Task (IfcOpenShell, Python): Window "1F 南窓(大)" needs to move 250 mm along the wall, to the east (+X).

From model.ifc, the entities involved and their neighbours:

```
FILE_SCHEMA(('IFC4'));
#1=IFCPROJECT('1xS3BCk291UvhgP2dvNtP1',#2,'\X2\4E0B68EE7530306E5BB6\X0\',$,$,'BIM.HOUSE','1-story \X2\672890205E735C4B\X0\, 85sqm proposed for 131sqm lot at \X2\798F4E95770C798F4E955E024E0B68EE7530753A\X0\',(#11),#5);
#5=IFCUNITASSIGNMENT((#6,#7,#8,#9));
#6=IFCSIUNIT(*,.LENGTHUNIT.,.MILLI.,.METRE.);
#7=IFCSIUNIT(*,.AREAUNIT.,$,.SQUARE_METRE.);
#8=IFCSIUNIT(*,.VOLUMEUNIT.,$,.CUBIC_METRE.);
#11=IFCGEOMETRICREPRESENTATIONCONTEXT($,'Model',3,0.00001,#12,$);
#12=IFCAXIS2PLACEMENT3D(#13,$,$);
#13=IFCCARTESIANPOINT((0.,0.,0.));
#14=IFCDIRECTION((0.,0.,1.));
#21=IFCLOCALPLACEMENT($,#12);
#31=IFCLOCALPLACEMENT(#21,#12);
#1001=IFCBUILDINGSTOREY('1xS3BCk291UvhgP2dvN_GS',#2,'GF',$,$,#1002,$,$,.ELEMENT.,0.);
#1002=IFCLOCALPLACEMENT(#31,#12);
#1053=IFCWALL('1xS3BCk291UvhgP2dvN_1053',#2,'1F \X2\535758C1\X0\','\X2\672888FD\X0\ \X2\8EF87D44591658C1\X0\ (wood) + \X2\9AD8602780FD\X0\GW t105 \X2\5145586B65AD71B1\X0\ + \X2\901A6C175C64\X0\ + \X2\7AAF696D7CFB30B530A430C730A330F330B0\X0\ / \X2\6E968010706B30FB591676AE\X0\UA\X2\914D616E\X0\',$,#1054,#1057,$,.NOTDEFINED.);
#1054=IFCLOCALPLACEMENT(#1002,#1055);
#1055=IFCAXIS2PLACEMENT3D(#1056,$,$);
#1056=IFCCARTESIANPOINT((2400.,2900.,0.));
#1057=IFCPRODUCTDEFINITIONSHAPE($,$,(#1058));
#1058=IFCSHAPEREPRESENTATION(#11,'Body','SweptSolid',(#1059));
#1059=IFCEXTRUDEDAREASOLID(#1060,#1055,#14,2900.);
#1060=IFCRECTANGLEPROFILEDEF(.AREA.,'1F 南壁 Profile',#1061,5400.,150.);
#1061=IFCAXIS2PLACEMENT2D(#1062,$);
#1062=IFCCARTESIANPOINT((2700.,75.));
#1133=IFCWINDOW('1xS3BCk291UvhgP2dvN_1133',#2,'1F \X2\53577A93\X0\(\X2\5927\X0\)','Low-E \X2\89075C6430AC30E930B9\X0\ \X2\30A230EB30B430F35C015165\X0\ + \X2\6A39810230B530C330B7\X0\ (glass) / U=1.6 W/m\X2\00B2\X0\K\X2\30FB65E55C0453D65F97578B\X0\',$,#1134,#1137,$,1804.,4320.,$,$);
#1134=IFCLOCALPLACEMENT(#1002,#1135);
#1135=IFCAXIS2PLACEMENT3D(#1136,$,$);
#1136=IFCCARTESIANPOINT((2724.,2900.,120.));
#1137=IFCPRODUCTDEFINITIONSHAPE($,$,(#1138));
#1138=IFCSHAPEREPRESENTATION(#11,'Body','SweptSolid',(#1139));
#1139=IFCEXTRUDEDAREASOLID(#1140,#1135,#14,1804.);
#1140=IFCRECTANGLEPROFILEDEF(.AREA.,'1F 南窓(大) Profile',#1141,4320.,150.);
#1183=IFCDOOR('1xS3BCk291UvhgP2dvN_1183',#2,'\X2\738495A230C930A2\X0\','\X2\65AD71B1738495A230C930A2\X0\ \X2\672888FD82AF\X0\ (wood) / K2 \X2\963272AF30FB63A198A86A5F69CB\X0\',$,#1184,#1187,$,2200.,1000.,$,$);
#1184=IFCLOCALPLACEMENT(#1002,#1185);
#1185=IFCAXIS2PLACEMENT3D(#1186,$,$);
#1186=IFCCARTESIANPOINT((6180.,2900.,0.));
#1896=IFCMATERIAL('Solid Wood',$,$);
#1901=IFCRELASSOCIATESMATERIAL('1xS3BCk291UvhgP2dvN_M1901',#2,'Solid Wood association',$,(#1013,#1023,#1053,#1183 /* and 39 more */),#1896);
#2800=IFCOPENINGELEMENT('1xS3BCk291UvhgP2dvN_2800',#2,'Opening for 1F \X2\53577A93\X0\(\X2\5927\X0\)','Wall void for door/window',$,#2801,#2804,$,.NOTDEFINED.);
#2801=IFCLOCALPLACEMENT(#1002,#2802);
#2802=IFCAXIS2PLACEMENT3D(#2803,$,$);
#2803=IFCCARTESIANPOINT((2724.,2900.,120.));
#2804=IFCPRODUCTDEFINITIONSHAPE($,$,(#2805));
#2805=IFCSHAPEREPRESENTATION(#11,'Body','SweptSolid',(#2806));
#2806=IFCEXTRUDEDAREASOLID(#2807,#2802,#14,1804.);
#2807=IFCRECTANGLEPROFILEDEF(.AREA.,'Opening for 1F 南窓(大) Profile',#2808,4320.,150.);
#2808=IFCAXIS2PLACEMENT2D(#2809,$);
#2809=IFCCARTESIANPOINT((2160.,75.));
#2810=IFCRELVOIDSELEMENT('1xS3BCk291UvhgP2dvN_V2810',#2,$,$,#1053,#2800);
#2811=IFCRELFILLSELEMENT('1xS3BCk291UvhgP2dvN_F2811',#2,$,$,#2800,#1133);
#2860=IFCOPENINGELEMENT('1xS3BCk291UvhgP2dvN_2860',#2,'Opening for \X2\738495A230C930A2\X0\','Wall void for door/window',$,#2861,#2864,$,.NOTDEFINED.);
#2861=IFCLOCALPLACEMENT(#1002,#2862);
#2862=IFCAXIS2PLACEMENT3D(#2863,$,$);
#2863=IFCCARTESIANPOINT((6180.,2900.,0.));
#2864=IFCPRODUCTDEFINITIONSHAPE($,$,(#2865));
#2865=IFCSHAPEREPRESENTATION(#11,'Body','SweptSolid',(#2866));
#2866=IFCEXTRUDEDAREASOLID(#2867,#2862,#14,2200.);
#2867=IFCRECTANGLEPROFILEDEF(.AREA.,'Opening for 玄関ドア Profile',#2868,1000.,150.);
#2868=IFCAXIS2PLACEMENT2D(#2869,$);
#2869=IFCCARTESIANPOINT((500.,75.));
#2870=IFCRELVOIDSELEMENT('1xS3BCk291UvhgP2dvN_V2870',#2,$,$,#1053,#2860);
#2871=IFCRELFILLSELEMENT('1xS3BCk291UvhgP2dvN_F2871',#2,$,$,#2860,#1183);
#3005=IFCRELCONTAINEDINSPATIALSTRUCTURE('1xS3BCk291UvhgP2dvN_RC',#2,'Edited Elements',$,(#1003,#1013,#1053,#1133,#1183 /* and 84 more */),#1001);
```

```python
import ifcopenshell
import ifcopenshell.api.geometry
import ifcopenshell.util.placement
import ifcopenshell.util.unit

model = ifcopenshell.open("model.ifc")
unit_scale = ifcopenshell.util.unit.calculate_unit_scale(model)

window = model.by_guid("1xS3BCk291UvhgP2dvN_1133")
opening = window.FillsVoids[0].RelatingOpeningElement
wall = opening.VoidsElements[0].RelatingBuildingElement

wall_matrix = ifcopenshell.util.placement.get_local_placement(wall.ObjectPlacement)
shift = wall_matrix[:3, 0] * 0.25 / unit_scale
before = ifcopenshell.util.placement.get_local_placement(window.ObjectPlacement)[:3, 3].copy()

# The window is not placed relative to its opening, so move both.
for product in (opening, window):
    matrix = ifcopenshell.util.placement.get_local_placement(product.ObjectPlacement)
    matrix[:3, 3] += shift
    ifcopenshell.api.geometry.edit_object_placement(model, product=product, matrix=matrix, is_si=False)

after = ifcopenshell.util.placement.get_local_placement(window.ObjectPlacement)[:3, 3]
print("window moved by", (after - before).round(3) + 0.0)

model.write("model_v2.ifc")
```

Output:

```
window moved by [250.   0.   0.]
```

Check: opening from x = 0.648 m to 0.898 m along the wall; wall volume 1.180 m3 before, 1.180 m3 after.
